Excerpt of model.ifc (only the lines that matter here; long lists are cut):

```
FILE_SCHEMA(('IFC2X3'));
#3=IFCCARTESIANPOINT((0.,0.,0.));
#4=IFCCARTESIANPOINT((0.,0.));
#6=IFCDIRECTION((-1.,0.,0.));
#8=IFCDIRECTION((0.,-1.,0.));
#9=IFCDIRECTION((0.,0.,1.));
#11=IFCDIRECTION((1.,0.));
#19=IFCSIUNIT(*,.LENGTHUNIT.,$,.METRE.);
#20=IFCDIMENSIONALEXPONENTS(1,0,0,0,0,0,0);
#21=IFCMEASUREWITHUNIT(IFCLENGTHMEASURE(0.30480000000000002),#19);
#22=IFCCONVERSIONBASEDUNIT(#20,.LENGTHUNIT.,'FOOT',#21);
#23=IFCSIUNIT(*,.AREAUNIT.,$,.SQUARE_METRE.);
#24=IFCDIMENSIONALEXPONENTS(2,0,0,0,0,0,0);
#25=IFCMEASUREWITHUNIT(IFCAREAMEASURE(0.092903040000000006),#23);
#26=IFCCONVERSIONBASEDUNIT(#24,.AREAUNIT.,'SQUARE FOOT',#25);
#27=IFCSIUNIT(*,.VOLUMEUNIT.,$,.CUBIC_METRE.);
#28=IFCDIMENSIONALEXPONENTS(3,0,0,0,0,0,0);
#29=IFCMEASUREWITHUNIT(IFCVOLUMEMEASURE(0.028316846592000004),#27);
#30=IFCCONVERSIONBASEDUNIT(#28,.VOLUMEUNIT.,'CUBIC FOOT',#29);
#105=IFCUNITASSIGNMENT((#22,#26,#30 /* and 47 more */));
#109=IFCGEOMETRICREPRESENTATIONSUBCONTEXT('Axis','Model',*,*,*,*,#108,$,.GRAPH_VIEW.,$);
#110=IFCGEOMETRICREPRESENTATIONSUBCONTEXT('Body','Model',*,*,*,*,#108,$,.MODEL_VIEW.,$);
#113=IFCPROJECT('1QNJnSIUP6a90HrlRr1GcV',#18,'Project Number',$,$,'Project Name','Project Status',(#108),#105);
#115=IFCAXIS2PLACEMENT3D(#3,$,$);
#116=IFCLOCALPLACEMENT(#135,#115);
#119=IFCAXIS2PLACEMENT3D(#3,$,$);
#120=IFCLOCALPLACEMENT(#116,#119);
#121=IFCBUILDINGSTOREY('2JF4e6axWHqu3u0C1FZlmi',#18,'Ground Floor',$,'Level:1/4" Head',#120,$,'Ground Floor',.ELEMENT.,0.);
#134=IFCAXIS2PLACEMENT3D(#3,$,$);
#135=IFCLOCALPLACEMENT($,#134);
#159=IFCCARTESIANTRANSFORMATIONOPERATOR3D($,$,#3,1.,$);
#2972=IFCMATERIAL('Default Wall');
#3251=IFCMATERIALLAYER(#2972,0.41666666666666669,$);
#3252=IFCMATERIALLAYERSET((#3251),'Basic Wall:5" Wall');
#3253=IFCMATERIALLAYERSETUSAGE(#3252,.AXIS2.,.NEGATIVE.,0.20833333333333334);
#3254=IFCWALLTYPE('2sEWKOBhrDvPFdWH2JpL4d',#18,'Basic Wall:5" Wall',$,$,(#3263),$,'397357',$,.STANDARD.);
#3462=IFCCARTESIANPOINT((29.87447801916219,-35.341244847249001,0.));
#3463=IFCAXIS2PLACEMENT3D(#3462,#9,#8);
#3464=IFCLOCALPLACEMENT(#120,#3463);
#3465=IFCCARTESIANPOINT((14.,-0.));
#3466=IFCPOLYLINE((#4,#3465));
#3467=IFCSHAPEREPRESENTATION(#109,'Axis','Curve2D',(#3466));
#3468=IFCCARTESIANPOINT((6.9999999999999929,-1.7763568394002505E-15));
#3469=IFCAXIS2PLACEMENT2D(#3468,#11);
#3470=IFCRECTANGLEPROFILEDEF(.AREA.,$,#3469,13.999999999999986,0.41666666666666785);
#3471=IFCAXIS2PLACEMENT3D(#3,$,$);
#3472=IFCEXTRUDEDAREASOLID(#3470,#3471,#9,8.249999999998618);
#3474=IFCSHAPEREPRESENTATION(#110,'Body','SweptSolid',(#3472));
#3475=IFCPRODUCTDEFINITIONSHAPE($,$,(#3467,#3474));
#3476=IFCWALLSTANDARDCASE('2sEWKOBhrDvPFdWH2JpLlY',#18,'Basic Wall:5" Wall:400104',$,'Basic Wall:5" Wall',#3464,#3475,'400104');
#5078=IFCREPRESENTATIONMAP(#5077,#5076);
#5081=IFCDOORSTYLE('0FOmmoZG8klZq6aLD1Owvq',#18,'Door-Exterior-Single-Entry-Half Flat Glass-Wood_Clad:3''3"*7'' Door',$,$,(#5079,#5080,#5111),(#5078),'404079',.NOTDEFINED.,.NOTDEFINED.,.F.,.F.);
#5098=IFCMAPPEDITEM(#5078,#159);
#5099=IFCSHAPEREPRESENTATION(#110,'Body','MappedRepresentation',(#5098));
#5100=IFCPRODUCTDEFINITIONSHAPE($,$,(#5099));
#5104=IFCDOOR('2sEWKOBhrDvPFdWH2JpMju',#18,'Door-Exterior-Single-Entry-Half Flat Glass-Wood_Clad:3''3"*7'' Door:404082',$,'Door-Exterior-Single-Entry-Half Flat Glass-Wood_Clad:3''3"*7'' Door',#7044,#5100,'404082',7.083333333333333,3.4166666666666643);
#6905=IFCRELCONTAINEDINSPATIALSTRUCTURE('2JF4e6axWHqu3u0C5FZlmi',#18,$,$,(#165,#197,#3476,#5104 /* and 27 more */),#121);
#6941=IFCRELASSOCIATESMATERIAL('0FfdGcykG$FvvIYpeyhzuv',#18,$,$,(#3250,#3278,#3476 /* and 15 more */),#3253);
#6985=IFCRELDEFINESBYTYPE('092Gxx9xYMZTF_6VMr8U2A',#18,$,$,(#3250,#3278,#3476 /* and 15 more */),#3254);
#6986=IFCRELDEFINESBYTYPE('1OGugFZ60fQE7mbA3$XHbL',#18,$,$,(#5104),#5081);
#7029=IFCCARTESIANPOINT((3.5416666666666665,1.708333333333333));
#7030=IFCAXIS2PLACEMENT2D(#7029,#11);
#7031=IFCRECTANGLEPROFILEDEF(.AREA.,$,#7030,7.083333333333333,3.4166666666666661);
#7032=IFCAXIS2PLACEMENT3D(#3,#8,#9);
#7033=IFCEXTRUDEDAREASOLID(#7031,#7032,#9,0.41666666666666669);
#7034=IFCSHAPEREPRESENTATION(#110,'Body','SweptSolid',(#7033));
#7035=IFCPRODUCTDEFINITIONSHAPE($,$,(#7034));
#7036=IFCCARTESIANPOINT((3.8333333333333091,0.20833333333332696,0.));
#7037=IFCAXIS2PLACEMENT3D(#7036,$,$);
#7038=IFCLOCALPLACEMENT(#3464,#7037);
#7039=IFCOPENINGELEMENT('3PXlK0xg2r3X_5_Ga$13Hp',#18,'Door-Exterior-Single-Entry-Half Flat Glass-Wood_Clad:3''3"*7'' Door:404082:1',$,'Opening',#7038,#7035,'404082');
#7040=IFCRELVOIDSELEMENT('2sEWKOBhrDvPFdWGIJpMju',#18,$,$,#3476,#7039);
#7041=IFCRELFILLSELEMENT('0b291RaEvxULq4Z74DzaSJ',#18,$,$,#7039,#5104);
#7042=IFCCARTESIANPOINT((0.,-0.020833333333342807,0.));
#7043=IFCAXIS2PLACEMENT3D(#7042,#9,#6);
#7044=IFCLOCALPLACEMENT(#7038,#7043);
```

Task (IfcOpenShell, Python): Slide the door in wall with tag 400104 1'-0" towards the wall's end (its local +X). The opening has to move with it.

```python
import ifcopenshell
import ifcopenshell.api.geometry
import ifcopenshell.util.placement
import ifcopenshell.util.unit

model = ifcopenshell.open("model.ifc")
unit_scale = ifcopenshell.util.unit.calculate_unit_scale(model)

door = model.by_guid("2sEWKOBhrDvPFdWH2JpMju")
opening = door.FillsVoids[0].RelatingOpeningElement
wall = opening.VoidsElements[0].RelatingBuildingElement

wall_matrix = ifcopenshell.util.placement.get_local_placement(wall.ObjectPlacement)
shift = wall_matrix[:3, 0] * 12 * 0.0254 / unit_scale
before = ifcopenshell.util.placement.get_local_placement(door.ObjectPlacement)[:3, 3].copy()

# The door is placed relative to its opening, so it follows when the opening moves.
matrix = ifcopenshell.util.placement.get_local_placement(opening.ObjectPlacement)
matrix[:3, 3] += shift
ifcopenshell.api.geometry.edit_object_placement(
    model, product=opening, matrix=matrix, is_si=False, should_transform_children=True
)

after = ifcopenshell.util.placement.get_local_placement(door.ObjectPlacement)[:3, 3]
print("door moved by", (after - before).round(3) + 0.0)

model.write("model_rev.ifc")
```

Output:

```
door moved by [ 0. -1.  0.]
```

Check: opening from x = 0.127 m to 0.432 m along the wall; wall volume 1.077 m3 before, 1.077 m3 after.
